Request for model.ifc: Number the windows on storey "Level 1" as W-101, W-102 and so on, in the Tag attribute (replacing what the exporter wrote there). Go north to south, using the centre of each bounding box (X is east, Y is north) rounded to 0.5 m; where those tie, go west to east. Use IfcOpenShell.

First a look at what the model holds.

```python
import ifcopenshell
import ifcopenshell.util.element
import ifcopenshell.util.placement

model = ifcopenshell.open("model.ifc")
print(model.schema)
storey = next(s for s in model.by_type("IfcBuildingStorey") if s.Name == "Level 1")
windows = [e for e in ifcopenshell.util.element.get_decomposition(storey) if e.is_a("IfcWindow")]
for e in sorted(windows, key=lambda e: e.id()):
    origin = ifcopenshell.util.placement.get_local_placement(e.ObjectPlacement)[:3, 3]
    print(e.id(), e.Tag, e.Name, origin.round(2) + 0.0, sep=" | ")
```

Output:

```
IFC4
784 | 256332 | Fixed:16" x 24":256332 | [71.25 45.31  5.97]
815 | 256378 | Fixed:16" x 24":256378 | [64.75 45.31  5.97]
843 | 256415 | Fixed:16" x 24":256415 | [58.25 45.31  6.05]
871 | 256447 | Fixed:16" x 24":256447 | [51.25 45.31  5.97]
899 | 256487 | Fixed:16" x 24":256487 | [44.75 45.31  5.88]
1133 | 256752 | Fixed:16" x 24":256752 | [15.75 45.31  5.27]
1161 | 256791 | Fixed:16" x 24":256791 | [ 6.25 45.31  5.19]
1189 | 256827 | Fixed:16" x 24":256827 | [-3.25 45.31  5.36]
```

```python
import ifcopenshell
import ifcopenshell.geom
import ifcopenshell.util.element
import ifcopenshell.util.shape

model = ifcopenshell.open("model.ifc")
settings = ifcopenshell.geom.settings()
settings.set("use-world-coords", True)


def centre(element):
    shape = ifcopenshell.geom.create_shape(settings, element)
    return ifcopenshell.util.shape.get_bbox_centroid(shape.geometry)


storey = next(s for s in model.by_type("IfcBuildingStorey") if s.Name == "Level 1")
windows = [e for e in ifcopenshell.util.element.get_decomposition(storey) if e.is_a("IfcWindow")]

# Insertion points can sit at a corner or the storey origin, so sort by the geometry (in metres).
centres = {e: centre(e) for e in windows}
windows.sort(key=lambda e: (-round(centres[e][1] / 0.5), centres[e][0]))

for i, e in enumerate(windows, start=1):
    number = f"W-1{i:02d}"
    e.Tag = number
    print(e.id(), number)

model.write("model_rev.ifc")
```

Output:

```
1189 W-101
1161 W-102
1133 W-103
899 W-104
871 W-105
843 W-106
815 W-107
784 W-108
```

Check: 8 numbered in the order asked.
